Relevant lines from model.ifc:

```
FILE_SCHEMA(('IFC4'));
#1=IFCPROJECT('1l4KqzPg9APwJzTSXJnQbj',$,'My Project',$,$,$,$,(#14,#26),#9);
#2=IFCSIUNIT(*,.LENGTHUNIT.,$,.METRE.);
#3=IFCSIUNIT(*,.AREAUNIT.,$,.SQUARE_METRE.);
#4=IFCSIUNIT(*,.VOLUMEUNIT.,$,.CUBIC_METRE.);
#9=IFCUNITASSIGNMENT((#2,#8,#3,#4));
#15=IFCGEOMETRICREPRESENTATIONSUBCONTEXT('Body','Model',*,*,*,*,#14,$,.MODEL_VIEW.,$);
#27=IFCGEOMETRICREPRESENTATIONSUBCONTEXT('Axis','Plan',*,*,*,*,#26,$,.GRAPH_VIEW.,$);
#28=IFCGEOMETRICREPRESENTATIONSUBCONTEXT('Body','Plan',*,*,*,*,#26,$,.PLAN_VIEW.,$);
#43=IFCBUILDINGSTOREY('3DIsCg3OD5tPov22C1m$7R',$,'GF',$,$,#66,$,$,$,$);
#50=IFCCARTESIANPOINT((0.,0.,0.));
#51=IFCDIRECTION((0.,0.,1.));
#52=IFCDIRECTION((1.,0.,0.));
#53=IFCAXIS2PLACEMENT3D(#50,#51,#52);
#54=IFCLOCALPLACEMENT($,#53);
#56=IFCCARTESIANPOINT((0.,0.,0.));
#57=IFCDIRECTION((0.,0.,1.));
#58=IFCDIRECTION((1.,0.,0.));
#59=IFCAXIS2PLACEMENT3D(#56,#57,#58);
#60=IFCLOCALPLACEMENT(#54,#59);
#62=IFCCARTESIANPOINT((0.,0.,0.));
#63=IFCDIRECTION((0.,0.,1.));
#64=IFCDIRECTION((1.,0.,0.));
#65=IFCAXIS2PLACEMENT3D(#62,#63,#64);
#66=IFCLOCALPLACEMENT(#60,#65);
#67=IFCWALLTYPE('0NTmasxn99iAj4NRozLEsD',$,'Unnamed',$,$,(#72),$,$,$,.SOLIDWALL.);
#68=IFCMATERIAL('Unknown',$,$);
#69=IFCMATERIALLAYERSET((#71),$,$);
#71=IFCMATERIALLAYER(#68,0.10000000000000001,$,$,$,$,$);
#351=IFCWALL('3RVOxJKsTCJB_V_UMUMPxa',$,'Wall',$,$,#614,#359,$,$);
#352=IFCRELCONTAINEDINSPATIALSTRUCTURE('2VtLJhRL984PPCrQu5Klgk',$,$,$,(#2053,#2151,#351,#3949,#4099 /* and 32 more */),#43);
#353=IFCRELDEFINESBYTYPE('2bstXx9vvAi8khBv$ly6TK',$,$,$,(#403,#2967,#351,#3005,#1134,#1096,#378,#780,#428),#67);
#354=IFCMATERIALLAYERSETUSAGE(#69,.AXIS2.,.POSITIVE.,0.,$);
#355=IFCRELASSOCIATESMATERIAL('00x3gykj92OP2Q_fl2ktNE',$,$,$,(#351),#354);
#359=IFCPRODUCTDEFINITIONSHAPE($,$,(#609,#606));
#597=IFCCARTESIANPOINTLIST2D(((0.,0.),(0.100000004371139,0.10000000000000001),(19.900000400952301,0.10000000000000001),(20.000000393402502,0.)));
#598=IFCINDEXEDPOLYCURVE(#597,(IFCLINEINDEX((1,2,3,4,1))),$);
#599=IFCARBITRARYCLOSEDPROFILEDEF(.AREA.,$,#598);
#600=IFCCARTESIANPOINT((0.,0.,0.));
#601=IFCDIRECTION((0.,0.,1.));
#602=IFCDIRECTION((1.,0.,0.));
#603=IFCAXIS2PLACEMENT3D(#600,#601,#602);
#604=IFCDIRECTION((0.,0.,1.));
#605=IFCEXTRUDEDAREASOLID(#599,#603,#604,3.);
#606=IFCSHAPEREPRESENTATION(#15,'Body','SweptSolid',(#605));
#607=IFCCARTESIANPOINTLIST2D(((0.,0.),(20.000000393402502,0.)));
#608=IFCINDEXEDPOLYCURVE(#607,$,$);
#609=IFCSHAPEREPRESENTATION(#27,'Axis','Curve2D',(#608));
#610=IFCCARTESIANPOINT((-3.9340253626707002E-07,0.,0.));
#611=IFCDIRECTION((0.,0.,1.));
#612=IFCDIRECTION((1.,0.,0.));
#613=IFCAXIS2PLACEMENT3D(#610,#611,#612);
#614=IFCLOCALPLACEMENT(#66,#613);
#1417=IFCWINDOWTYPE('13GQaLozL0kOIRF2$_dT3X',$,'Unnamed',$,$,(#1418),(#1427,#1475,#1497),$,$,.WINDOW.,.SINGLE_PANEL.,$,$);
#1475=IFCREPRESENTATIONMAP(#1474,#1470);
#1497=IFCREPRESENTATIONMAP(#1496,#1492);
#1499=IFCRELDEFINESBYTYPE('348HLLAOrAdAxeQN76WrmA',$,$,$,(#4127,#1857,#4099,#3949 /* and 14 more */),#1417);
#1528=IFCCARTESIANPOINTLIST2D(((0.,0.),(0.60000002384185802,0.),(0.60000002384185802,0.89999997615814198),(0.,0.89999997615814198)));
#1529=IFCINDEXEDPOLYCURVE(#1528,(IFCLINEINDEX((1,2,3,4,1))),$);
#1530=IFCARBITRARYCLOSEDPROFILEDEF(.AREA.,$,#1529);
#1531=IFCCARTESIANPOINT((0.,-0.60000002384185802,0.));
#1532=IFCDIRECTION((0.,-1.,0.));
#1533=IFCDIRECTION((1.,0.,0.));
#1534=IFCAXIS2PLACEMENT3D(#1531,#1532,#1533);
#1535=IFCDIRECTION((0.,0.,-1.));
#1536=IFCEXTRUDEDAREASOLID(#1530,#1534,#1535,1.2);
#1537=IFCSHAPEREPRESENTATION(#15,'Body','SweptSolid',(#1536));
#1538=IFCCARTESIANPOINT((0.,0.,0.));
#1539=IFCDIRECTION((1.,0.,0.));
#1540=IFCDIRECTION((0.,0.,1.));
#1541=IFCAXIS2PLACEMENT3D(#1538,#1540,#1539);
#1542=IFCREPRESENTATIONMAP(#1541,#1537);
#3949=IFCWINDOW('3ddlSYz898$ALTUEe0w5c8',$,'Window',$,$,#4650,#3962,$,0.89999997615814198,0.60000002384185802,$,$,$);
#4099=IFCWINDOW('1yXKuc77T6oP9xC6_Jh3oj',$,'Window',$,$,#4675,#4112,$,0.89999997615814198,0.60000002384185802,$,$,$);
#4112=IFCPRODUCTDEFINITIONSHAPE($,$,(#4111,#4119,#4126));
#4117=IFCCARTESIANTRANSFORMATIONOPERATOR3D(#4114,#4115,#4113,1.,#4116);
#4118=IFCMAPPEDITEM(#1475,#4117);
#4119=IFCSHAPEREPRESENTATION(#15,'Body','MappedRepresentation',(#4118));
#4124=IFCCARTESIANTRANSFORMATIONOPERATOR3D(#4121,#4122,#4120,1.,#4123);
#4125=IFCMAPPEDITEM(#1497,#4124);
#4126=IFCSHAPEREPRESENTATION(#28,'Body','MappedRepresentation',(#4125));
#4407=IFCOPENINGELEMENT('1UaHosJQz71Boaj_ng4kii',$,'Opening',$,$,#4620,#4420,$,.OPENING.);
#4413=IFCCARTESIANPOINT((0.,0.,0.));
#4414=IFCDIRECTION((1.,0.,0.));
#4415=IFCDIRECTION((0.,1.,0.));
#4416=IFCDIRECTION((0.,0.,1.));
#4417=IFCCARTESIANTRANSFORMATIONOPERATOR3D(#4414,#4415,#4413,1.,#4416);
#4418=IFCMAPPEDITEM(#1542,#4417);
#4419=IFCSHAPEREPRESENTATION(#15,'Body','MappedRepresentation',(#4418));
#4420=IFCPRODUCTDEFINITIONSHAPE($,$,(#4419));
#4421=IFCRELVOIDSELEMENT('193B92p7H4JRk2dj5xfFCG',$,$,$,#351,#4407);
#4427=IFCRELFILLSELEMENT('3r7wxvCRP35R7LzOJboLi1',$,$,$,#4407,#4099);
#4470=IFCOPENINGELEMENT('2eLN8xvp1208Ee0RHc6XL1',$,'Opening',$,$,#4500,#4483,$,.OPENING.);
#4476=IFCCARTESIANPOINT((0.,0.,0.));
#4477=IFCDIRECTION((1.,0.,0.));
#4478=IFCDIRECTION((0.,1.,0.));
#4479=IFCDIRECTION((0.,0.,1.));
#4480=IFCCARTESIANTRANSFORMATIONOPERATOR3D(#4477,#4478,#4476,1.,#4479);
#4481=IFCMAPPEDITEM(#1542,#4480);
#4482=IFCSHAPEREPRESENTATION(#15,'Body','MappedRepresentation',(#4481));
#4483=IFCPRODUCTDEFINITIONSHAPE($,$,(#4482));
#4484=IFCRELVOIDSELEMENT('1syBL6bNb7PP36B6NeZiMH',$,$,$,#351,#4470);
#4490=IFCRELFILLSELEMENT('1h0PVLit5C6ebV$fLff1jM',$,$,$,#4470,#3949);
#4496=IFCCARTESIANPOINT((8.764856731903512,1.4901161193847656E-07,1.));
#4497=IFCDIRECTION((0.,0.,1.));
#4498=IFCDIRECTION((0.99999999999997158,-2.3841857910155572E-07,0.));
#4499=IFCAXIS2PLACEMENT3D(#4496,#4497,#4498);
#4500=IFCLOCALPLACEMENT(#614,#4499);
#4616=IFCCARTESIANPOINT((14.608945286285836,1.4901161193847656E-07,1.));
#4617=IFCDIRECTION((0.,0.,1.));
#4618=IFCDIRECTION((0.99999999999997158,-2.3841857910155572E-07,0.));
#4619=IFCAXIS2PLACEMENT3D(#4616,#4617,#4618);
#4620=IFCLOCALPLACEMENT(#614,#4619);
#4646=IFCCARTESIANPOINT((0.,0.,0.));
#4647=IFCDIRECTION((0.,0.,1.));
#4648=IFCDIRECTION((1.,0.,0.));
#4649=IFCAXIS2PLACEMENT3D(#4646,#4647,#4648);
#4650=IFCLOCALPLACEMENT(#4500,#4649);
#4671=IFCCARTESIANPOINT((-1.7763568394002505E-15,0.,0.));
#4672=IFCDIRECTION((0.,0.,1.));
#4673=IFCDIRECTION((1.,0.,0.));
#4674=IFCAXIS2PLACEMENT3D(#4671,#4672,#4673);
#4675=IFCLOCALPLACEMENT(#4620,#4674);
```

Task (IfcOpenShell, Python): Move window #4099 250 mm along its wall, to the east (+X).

```python
import ifcopenshell
import ifcopenshell.api.geometry
import ifcopenshell.util.placement

model = ifcopenshell.open("model.ifc")

window = model.by_guid("1yXKuc77T6oP9xC6_Jh3oj")
opening = window.FillsVoids[0].RelatingOpeningElement
wall = opening.VoidsElements[0].RelatingBuildingElement

wall_matrix = ifcopenshell.util.placement.get_local_placement(wall.ObjectPlacement)
shift = wall_matrix[:3, 0] * 0.25
before = ifcopenshell.util.placement.get_local_placement(window.ObjectPlacement)[:3, 3].copy()

# The window is placed relative to its opening, so it follows when the opening moves.
matrix = ifcopenshell.util.placement.get_local_placement(opening.ObjectPlacement)
matrix[:3, 3] += shift
ifcopenshell.api.geometry.edit_object_placement(
    model, product=opening, matrix=matrix, is_si=False, should_transform_children=True
)

after = ifcopenshell.util.placement.get_local_placement(window.ObjectPlacement)[:3, 3]
print("window moved by", (after - before).round(3) + 0.0)

model.write("model_v2.ifc")
```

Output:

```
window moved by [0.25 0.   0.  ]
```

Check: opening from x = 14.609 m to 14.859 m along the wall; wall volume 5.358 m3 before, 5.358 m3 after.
